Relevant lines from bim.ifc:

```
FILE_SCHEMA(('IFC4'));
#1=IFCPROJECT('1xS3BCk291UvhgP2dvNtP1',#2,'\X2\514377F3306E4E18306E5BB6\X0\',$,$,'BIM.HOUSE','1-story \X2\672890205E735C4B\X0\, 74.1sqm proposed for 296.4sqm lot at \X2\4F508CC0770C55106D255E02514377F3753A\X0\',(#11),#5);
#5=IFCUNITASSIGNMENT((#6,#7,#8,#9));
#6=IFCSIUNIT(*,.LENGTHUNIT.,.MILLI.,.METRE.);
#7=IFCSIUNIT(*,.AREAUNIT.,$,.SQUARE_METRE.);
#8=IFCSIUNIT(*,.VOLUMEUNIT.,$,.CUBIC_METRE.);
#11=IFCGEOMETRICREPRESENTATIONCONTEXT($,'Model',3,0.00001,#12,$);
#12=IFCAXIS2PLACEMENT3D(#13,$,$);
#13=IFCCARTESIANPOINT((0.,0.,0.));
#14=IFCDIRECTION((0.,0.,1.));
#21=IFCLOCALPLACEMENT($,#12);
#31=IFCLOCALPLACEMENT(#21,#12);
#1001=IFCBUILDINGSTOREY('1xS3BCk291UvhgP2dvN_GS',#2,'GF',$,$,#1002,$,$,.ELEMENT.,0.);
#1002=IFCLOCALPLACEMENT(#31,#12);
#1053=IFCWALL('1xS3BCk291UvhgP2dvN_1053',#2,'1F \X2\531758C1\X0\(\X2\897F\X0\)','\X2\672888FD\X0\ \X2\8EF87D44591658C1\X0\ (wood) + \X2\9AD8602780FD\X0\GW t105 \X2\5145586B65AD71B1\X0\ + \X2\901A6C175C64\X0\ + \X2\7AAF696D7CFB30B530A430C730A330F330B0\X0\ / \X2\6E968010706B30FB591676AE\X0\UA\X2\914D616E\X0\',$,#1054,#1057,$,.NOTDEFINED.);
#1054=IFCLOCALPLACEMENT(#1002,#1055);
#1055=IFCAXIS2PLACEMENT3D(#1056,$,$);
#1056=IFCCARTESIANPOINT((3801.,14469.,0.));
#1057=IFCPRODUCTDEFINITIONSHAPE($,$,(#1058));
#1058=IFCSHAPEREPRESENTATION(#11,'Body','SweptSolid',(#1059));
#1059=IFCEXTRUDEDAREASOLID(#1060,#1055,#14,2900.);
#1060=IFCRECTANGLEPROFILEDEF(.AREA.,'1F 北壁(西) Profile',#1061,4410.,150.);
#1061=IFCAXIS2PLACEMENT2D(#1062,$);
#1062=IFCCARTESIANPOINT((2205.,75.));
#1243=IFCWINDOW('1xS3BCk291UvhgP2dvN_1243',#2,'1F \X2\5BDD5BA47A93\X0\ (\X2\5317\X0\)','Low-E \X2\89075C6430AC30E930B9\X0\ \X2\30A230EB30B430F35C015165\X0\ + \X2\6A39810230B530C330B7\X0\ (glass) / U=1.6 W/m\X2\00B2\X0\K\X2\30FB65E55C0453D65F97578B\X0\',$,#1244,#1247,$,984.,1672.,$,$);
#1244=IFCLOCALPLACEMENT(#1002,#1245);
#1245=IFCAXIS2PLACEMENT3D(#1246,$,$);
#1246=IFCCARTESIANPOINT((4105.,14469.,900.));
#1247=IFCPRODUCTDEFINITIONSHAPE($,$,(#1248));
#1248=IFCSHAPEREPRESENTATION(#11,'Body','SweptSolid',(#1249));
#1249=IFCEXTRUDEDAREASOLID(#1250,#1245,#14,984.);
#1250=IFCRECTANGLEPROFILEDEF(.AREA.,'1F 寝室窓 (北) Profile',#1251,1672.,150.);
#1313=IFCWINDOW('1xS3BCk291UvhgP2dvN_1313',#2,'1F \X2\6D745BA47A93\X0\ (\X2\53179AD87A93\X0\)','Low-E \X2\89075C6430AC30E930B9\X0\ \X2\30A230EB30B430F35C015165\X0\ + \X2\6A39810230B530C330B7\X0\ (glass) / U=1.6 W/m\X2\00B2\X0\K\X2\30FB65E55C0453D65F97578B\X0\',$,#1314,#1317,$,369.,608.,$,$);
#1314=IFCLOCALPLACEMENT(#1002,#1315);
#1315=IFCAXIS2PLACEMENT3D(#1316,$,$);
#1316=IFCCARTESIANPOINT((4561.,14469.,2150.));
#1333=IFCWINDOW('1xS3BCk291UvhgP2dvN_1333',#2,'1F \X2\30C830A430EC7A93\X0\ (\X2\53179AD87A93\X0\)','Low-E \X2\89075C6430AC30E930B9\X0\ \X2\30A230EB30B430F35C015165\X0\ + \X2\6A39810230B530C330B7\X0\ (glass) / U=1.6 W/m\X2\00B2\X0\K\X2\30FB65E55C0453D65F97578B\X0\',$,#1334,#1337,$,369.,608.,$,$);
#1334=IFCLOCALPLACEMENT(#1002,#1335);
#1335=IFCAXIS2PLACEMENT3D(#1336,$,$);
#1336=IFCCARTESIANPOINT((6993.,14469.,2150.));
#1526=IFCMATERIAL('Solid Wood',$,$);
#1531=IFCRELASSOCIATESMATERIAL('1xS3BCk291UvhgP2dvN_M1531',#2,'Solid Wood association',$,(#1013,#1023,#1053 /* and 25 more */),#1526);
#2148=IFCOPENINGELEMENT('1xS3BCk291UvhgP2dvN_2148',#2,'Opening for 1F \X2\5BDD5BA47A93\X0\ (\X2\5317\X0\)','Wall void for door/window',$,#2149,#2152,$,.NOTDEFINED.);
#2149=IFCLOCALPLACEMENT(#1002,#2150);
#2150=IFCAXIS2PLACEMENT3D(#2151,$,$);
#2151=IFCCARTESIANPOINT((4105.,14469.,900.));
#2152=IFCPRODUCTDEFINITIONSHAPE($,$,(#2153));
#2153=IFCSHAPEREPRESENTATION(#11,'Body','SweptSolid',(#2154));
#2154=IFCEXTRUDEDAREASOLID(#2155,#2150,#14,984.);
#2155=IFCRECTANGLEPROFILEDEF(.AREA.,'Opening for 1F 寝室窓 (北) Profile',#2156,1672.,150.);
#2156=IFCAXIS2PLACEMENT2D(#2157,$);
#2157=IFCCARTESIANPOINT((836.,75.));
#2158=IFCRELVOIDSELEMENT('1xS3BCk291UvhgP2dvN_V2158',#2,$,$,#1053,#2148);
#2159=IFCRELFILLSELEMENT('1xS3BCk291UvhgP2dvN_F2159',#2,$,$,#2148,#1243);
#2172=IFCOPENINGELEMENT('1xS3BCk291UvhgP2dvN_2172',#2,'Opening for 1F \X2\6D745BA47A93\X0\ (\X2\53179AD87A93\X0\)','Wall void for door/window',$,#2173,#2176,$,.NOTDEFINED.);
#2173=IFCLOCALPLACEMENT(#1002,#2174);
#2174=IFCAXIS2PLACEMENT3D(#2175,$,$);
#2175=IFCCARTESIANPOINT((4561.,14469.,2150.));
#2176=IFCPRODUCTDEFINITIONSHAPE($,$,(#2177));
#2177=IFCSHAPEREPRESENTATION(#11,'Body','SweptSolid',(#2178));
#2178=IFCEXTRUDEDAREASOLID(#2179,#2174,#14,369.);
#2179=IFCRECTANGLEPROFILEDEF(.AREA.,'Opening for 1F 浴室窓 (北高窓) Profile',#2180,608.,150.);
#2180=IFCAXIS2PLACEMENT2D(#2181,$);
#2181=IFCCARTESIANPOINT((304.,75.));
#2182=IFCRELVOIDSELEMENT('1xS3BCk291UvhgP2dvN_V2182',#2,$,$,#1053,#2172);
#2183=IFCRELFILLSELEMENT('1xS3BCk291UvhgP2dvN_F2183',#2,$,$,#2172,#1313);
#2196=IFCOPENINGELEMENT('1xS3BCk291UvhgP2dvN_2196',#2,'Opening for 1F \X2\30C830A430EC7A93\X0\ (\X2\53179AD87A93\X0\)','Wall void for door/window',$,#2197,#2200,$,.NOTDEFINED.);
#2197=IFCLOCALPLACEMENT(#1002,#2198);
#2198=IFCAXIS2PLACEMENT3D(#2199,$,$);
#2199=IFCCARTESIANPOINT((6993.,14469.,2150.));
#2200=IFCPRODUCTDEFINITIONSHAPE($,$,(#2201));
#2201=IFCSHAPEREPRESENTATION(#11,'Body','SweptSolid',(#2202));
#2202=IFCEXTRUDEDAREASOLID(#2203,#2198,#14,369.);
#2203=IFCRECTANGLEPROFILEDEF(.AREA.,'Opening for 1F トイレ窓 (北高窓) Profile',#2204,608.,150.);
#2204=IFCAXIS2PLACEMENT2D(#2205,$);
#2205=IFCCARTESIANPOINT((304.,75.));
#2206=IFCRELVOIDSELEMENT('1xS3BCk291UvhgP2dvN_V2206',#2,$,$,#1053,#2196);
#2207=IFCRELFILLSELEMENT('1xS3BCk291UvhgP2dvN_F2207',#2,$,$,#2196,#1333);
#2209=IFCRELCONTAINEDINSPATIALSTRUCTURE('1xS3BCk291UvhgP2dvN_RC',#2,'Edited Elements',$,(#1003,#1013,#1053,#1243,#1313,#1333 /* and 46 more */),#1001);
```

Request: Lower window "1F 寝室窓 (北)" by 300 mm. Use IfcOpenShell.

```python
import numpy as np
import ifcopenshell
import ifcopenshell.api.geometry
import ifcopenshell.util.placement
import ifcopenshell.util.unit

model = ifcopenshell.open("bim.ifc")
unit_scale = ifcopenshell.util.unit.calculate_unit_scale(model)

window = model.by_guid("1xS3BCk291UvhgP2dvN_1243")
opening = window.FillsVoids[0].RelatingOpeningElement
dz = -0.3 / unit_scale

shift = np.array([0.0, 0.0, dz])
# The window is not placed relative to its opening, so move both.
for product in (opening, window):
    matrix = ifcopenshell.util.placement.get_local_placement(product.ObjectPlacement)
    matrix[:3, 3] += shift
    ifcopenshell.api.geometry.edit_object_placement(model, product=product, matrix=matrix, is_si=False)

print(f"moved by {dz * unit_scale:+.3f} m")

model.write("bim-out.ifc")
```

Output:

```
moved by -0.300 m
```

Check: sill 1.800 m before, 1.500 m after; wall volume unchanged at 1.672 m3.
